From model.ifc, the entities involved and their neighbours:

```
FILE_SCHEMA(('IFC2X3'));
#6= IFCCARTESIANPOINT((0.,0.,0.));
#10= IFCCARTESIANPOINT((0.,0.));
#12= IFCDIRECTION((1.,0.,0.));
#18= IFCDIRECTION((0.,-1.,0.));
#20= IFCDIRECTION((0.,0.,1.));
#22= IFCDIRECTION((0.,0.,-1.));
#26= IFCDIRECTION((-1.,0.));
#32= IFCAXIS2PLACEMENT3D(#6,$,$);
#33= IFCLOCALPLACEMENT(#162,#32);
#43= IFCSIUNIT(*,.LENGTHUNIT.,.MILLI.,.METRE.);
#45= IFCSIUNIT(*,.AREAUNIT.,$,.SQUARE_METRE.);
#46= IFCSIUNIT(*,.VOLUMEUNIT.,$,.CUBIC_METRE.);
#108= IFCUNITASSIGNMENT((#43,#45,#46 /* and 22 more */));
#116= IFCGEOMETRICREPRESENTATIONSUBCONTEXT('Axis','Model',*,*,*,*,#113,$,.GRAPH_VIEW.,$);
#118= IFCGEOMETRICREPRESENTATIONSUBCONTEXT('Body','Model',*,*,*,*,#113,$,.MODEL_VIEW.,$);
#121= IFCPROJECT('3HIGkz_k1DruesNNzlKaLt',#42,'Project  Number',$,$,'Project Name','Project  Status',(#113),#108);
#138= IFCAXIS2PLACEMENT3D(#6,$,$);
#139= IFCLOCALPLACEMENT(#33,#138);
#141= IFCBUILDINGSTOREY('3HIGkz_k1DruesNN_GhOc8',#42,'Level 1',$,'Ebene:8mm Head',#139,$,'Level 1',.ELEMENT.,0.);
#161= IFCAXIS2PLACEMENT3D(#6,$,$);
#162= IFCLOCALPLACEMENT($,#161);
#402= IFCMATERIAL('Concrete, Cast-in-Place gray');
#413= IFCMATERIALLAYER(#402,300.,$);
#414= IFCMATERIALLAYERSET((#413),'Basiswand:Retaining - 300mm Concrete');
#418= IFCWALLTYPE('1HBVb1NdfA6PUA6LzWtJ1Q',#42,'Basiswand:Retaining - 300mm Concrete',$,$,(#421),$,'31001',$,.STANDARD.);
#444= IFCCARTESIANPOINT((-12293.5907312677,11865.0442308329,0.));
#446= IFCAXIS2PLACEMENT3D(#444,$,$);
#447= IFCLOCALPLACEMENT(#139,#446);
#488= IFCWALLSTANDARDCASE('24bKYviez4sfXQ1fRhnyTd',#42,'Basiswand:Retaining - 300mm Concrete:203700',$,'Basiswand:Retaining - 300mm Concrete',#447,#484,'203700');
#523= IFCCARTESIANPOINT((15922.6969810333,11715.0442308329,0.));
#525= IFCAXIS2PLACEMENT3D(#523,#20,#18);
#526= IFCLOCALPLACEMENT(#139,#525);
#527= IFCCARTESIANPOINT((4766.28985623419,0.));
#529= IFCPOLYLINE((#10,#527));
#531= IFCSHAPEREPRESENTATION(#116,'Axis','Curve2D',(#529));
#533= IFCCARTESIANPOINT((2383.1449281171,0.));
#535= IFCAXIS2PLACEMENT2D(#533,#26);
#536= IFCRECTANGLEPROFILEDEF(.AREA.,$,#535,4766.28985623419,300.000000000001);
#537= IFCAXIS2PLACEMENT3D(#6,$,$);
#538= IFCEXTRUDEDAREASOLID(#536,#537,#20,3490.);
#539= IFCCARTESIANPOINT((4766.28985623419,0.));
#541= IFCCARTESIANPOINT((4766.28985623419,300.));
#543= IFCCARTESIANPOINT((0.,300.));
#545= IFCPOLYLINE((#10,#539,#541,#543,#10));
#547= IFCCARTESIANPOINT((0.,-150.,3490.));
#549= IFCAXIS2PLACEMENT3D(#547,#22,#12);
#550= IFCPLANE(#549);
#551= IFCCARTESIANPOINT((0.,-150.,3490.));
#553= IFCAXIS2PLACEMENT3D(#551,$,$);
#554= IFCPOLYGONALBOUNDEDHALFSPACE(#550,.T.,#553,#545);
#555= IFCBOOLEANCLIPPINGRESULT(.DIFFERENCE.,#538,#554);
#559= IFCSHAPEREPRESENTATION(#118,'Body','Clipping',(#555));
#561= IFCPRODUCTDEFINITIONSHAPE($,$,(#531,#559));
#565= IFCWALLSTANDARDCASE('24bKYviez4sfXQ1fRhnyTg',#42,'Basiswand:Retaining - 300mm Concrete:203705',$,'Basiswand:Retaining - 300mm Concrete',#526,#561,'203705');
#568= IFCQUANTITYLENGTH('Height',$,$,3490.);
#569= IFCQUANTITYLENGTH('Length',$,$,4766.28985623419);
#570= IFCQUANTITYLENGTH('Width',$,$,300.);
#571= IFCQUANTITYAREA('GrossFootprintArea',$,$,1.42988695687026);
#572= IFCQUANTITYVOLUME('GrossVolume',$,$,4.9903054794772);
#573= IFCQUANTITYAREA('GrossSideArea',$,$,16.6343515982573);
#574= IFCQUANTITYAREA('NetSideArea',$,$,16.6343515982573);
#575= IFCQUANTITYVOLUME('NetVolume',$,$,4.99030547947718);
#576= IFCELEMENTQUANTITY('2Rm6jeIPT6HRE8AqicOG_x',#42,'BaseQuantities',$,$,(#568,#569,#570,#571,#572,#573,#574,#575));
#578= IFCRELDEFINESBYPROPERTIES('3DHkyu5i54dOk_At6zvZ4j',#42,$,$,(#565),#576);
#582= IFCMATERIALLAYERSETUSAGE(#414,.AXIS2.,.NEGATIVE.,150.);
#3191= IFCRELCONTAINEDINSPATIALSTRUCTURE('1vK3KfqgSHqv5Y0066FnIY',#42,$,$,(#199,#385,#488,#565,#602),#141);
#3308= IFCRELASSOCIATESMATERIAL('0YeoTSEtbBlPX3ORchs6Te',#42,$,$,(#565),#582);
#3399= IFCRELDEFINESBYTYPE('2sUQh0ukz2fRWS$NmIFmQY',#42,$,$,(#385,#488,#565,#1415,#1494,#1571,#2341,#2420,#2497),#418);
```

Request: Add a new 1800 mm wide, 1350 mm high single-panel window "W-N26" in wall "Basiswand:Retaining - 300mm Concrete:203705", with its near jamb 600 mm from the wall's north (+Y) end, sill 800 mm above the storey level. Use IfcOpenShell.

```python
import numpy as np
import ifcopenshell
import ifcopenshell.api.feature
import ifcopenshell.api.geometry
import ifcopenshell.api.pset
import ifcopenshell.api.root
import ifcopenshell.api.spatial
import ifcopenshell.api.type
import ifcopenshell.geom
import ifcopenshell.util.element
import ifcopenshell.util.placement
import ifcopenshell.util.representation
import ifcopenshell.util.shape
import ifcopenshell.util.unit

model = ifcopenshell.open("model.ifc")
unit_scale = ifcopenshell.util.unit.calculate_unit_scale(model)
area_scale = ifcopenshell.util.unit.calculate_unit_scale(model, "AREAUNIT")
volume_scale = ifcopenshell.util.unit.calculate_unit_scale(model, "VOLUMEUNIT")
settings = ifcopenshell.geom.settings()


def volume(element):
    """Net volume in cubic metres, openings subtracted."""
    shape = ifcopenshell.geom.create_shape(settings, element)
    return ifcopenshell.util.shape.get_volume(shape.geometry)


wall = model.by_guid("24bKYviez4sfXQ1fRhnyTg")
storey = ifcopenshell.util.element.get_container(wall, ifc_class="IfcBuildingStorey")
context = ifcopenshell.util.representation.get_context(model, "Model", "Body", "MODEL_VIEW")
before = volume(wall)

width, height, from_end, sill = 1.8, 1.35, 0.6, 0.8  # metres

# The wall runs along its own X axis, and the end named is its -X end.
wall_shape = ifcopenshell.geom.create_shape(settings, wall)
x, y, z = ifcopenshell.util.shape.get_vertices(wall_shape.geometry).T
start = x.min() + from_end
face, thickness = float(y.min()), float(y.max() - y.min())
wall_matrix = ifcopenshell.util.placement.get_local_placement(wall.ObjectPlacement)
level = ifcopenshell.util.placement.get_local_placement(storey.ObjectPlacement)[2, 3]


def in_wall(x, y):
    """Placement at x, y metres in the wall's axes, at sill height."""
    matrix = wall_matrix.copy()
    matrix[:, 3] = wall_matrix @ np.array([x / unit_scale, y / unit_scale, 0.0, 1.0])
    matrix[2, 3] = level + sill / unit_scale
    return matrix


# Opening: a box that overshoots both wall faces by 50 mm.
opening = ifcopenshell.api.root.create_entity(model, ifc_class="IfcOpeningElement")
box = ifcopenshell.api.geometry.add_wall_representation(
    model, context=context, length=width, height=height, thickness=thickness + 0.1
)
ifcopenshell.api.geometry.assign_representation(model, product=opening, representation=box)
ifcopenshell.api.geometry.edit_object_placement(model, product=opening, matrix=in_wall(start, face - 0.05), is_si=False)
ifcopenshell.api.feature.add_feature(model, feature=opening, element=wall)

window = ifcopenshell.api.root.create_entity(model, ifc_class="IfcWindow", name="W-N26")
window.OverallWidth, window.OverallHeight = width / unit_scale, height / unit_scale
body = ifcopenshell.api.geometry.add_window_representation(
    model,
    context=context,
    overall_width=window.OverallWidth,
    overall_height=window.OverallHeight,
    partition_type="SINGLE_PANEL",
)
ifcopenshell.api.geometry.assign_representation(model, product=window, representation=body)
ifcopenshell.api.spatial.assign_container(model, products=[window], relating_structure=storey)
fills = ifcopenshell.api.feature.add_filling(model, opening=opening, element=window)
fills.OwnerHistory = window.OwnerHistory  # required in IFC2X3

# IFC2X3 keeps the operation on the window style.
style = ifcopenshell.api.root.create_entity(model, ifc_class="IfcWindowStyle", name="W-N26")
style.OperationType, style.ConstructionType = "SINGLE_PANEL", "NOTDEFINED"
style.ParameterTakesPrecedence = style.Sizeable = False
ifcopenshell.api.type.assign_type(model, related_objects=[window], relating_type=style)

# Centre the window in the wall's thickness.
ifcopenshell.api.geometry.edit_object_placement(model, product=window, matrix=in_wall(start, face), is_si=False)
window_shape = ifcopenshell.geom.create_shape(settings, window)
depth = ifcopenshell.util.shape.get_vertices(window_shape.geometry)[:, 1]
offset = face + thickness / 2 - (depth.min() + depth.max()) / 2
ifcopenshell.api.geometry.edit_object_placement(model, product=window, matrix=in_wall(start, offset), is_si=False)

after = volume(wall)

# Update the wall's stored quantities.
qto = model.by_id(ifcopenshell.util.element.get_pset(wall, "BaseQuantities", should_inherit=False)["id"])
ifcopenshell.api.pset.edit_qto(model, qto=qto, properties={
    "NetSideArea": after / thickness / area_scale,
    "NetVolume": after / volume_scale,
})

print(f"wall volume {before:.3f} -> {after:.3f} m3")

model.write("model-out.ifc")
```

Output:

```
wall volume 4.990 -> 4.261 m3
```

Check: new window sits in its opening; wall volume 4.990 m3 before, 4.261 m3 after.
